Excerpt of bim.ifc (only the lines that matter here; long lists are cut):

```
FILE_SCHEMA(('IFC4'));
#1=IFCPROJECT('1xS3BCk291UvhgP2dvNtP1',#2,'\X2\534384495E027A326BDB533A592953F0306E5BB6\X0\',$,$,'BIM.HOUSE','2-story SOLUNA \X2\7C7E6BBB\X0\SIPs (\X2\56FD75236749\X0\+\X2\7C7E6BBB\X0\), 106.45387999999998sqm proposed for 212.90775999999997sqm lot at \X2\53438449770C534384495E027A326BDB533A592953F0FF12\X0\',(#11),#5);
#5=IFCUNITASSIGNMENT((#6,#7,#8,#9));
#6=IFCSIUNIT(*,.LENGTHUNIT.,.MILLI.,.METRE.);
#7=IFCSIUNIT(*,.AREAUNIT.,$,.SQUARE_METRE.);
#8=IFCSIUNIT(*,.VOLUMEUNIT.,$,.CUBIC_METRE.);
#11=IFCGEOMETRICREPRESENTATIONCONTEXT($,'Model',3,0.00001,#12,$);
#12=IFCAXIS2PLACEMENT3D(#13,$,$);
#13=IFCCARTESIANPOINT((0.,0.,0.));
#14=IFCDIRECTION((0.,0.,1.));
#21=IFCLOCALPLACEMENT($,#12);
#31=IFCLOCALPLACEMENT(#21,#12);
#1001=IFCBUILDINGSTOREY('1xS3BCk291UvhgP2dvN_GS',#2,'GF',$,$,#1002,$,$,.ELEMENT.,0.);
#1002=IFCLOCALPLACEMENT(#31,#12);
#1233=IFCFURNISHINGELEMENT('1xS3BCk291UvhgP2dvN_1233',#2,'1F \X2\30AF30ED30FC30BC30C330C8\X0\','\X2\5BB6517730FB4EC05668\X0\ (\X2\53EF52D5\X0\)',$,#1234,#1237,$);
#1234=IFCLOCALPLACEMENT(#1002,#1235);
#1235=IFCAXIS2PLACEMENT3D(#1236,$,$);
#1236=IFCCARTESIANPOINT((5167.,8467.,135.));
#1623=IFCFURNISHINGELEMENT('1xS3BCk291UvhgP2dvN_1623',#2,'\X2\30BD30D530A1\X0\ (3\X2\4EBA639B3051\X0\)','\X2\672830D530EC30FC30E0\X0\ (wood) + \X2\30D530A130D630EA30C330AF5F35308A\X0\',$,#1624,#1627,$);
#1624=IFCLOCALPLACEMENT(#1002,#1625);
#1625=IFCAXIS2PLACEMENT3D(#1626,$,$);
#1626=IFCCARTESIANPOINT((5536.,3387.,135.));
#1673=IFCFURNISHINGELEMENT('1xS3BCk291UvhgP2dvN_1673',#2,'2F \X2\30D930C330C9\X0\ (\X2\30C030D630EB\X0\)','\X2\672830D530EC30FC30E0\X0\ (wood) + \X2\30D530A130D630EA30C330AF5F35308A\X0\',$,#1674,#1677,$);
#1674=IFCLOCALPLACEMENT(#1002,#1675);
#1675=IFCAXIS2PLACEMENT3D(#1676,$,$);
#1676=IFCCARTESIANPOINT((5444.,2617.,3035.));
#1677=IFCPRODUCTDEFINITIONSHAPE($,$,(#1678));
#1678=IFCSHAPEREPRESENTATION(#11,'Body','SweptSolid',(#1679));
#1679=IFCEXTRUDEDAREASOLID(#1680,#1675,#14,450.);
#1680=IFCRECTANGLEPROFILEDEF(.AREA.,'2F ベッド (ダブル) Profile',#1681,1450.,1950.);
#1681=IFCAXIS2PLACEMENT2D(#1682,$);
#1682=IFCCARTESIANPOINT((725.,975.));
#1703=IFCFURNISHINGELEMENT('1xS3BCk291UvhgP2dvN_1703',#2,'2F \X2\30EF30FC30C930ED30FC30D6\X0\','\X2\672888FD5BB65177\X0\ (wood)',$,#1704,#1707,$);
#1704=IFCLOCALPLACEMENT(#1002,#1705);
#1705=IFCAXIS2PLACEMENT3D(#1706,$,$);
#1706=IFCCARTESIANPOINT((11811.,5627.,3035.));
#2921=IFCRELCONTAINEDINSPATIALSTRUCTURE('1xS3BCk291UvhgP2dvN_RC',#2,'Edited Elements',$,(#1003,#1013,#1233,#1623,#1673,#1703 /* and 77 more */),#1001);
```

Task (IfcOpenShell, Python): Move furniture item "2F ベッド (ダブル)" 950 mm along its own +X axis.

```python
import ifcopenshell
import ifcopenshell.api.geometry
import ifcopenshell.util.placement

model = ifcopenshell.open("bim.ifc")

item = model.by_id(1673)
matrix = ifcopenshell.util.placement.get_local_placement(item.ObjectPlacement)
matrix[:3, 3] += matrix[:3, 0] * 950.0
ifcopenshell.api.geometry.edit_object_placement(model, product=item, matrix=matrix, is_si=False)

print(ifcopenshell.util.placement.get_local_placement(item.ObjectPlacement).round(3) + 0.0)

model.write("bim_v2.ifc")
```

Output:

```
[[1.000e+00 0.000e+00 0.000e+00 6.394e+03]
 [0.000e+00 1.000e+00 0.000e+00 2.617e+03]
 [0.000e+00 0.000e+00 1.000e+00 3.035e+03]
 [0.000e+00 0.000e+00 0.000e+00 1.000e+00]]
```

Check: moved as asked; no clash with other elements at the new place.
